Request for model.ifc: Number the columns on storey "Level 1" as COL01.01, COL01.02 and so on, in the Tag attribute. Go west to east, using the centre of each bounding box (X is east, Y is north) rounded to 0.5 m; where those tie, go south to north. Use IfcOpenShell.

First a look at what the model holds.

```python
import ifcopenshell
import ifcopenshell.util.element
import ifcopenshell.util.placement

model = ifcopenshell.open("model.ifc")
print(model.schema)
storey = next(s for s in model.by_type("IfcBuildingStorey") if s.Name == "Level 1")
columns = [e for e in ifcopenshell.util.element.get_decomposition(storey) if e.is_a("IfcColumn")]
for e in sorted(columns, key=lambda e: e.id()):
    origin = ifcopenshell.util.placement.get_local_placement(e.ObjectPlacement)[:3, 3]
    print(e.id(), e.Tag, e.Name, origin.round(2) + 0.0, sep=" | ")
```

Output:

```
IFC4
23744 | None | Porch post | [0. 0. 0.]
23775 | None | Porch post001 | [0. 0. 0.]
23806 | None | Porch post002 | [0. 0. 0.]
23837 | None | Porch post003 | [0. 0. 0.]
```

```python
import ifcopenshell
import ifcopenshell.geom
import ifcopenshell.util.element
import ifcopenshell.util.shape

model = ifcopenshell.open("model.ifc")
settings = ifcopenshell.geom.settings()
settings.set("use-world-coords", True)


def centre(element):
    shape = ifcopenshell.geom.create_shape(settings, element)
    return ifcopenshell.util.shape.get_bbox_centroid(shape.geometry)


storey = next(s for s in model.by_type("IfcBuildingStorey") if s.Name == "Level 1")
columns = [e for e in ifcopenshell.util.element.get_decomposition(storey) if e.is_a("IfcColumn")]

# Insertion points can sit at a corner or the storey origin, so sort by the geometry (in metres).
centres = {e: centre(e) for e in columns}
columns.sort(key=lambda e: (round(centres[e][0] / 0.5), centres[e][1]))

for i, e in enumerate(columns, start=1):
    number = f"COL01.{i:02d}"
    e.Tag = number
    print(e.id(), number)

model.write("model-out.ifc")
```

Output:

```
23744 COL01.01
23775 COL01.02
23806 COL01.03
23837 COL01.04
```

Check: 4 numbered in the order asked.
